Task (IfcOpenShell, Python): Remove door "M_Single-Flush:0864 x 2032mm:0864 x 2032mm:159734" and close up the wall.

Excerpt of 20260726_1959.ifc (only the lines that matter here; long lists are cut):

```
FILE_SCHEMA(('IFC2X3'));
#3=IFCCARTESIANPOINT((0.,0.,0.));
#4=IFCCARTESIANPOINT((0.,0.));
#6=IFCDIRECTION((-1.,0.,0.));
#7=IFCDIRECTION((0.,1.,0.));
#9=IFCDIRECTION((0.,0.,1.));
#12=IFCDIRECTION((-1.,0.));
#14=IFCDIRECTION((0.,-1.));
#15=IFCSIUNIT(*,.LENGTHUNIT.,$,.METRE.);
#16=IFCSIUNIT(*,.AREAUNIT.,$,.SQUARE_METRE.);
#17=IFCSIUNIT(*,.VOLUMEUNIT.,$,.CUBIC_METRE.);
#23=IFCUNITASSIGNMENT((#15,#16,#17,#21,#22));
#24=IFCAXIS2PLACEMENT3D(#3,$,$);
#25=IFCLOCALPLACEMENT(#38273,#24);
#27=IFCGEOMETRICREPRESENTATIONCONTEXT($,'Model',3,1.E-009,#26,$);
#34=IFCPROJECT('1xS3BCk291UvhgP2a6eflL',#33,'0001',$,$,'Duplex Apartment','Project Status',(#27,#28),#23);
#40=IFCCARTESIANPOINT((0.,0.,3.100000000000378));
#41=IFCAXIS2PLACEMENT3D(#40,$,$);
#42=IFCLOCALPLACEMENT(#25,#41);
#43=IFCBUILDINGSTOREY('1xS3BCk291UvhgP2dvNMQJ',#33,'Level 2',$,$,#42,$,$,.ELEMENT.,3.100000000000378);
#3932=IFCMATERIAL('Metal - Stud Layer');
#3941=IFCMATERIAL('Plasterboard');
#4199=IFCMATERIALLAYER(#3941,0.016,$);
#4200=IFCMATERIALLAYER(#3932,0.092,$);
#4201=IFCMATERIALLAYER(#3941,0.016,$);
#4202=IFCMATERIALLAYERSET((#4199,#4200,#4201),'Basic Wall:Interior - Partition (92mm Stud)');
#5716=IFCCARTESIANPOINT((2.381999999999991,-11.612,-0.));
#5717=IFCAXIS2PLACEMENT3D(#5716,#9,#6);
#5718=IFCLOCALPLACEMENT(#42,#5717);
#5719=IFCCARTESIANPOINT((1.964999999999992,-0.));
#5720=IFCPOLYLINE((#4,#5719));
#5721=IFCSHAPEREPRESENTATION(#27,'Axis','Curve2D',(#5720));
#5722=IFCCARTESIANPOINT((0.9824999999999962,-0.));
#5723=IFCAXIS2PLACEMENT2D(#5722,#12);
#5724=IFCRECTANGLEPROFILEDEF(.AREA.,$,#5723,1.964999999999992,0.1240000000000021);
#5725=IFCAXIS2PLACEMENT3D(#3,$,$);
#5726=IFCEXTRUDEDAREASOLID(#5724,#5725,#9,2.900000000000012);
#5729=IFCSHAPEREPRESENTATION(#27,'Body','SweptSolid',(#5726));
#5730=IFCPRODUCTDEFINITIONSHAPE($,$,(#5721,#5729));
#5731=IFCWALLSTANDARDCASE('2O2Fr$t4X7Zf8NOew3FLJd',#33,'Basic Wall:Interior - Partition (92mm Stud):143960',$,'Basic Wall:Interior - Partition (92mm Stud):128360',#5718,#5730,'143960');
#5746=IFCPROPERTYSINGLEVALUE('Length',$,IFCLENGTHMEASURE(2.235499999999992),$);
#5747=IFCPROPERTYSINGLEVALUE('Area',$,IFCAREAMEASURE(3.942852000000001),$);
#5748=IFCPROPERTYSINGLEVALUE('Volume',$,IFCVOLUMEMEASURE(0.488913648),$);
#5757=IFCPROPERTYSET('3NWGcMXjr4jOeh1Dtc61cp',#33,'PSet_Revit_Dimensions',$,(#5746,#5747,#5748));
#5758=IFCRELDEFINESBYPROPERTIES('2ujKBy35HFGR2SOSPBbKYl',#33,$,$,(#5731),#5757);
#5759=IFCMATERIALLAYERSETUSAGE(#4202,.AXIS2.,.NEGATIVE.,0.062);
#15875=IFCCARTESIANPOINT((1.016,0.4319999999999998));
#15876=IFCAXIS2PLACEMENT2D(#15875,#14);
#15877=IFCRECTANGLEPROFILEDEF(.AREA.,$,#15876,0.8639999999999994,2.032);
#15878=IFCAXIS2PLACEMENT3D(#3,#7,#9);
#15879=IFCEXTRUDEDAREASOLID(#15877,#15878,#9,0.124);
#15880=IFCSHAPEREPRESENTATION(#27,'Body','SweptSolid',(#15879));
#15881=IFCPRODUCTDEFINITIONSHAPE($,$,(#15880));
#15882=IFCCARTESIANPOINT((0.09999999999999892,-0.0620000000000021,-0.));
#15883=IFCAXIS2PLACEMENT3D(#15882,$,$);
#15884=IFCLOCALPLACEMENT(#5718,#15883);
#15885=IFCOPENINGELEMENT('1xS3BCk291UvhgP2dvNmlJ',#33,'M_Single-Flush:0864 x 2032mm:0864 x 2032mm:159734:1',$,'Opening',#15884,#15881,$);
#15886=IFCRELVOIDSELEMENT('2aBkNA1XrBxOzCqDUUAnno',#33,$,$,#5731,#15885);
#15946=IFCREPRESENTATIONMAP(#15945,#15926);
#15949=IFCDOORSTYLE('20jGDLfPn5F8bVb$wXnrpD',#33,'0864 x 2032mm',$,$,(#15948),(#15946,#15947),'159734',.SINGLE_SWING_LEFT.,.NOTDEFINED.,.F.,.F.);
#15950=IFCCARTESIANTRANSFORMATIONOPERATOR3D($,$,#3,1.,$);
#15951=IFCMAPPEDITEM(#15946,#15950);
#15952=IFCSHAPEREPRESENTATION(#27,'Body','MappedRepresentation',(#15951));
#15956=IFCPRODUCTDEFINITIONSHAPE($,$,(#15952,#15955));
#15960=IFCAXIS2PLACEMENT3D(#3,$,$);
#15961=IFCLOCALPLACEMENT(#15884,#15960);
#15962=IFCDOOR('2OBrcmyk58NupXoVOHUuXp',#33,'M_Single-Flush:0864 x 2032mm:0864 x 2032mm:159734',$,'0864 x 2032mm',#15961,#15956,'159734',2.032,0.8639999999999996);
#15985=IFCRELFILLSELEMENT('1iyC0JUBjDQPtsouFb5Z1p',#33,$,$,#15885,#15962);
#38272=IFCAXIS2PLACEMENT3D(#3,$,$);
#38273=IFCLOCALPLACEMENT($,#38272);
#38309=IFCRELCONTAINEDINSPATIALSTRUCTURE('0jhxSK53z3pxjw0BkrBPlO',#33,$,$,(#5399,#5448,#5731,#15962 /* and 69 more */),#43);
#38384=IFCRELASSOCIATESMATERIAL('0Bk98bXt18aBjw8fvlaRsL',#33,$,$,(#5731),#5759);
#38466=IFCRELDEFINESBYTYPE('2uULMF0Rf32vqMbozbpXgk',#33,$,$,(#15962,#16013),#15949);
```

```python
import ifcopenshell
import ifcopenshell.api.feature
import ifcopenshell.api.pset
import ifcopenshell.api.root
import ifcopenshell.geom
import ifcopenshell.util.element
import ifcopenshell.util.shape
import ifcopenshell.util.unit

model = ifcopenshell.open("20260726_1959.ifc")
area_scale = ifcopenshell.util.unit.calculate_unit_scale(model, "AREAUNIT")
volume_scale = ifcopenshell.util.unit.calculate_unit_scale(model, "VOLUMEUNIT")
settings = ifcopenshell.geom.settings()


def volume(element):
    """Net volume in cubic metres, openings subtracted."""
    shape = ifcopenshell.geom.create_shape(settings, element)
    return ifcopenshell.util.shape.get_volume(shape.geometry)


door = model.by_id(15962)
opening = door.FillsVoids[0].RelatingOpeningElement
wall = opening.VoidsElements[0].RelatingBuildingElement
before = volume(wall)

ifcopenshell.api.root.remove_product(model, product=door)
ifcopenshell.api.feature.remove_feature(model, feature=opening)

after = volume(wall)
thickness = 0.124  # wall thickness in metres

# Update the wall's stored quantities.
pset = model.by_id(ifcopenshell.util.element.get_pset(wall, "PSet_Revit_Dimensions", should_inherit=False)["id"])
ifcopenshell.api.pset.edit_pset(model, pset=pset, properties={
    "Area": model.create_entity("IfcAreaMeasure", after / thickness / area_scale),
    "Volume": model.create_entity("IfcVolumeMeasure", after / volume_scale),
})

print(f"wall volume {before:.3f} -> {after:.3f} m3")

model.write("20260726_1959-out.ifc")
```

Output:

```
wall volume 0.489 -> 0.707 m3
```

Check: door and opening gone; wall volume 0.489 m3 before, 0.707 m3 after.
